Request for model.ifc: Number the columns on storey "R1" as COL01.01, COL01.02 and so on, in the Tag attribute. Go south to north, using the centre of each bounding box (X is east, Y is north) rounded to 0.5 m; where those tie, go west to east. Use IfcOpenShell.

First a look at what the model holds.

```python
import ifcopenshell
import ifcopenshell.util.element
import ifcopenshell.util.placement

model = ifcopenshell.open("model.ifc")
print(model.schema)
storey = next(s for s in model.by_type("IfcBuildingStorey") if s.Name == "R1")
columns = [e for e in ifcopenshell.util.element.get_decomposition(storey) if e.is_a("IfcColumn")]
for e in sorted(columns, key=lambda e: e.id()):
    origin = ifcopenshell.util.placement.get_local_placement(e.ObjectPlacement)[:3, 3]
    print(e.id(), e.Tag, e.Name, origin.round(2) + 0.0, sep=" | ")
```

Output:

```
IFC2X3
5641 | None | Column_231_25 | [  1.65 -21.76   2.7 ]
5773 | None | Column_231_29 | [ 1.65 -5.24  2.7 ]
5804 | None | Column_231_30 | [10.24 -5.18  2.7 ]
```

```python
import ifcopenshell
import ifcopenshell.geom
import ifcopenshell.util.element
import ifcopenshell.util.shape

model = ifcopenshell.open("model.ifc")
settings = ifcopenshell.geom.settings()
settings.set("use-world-coords", True)


def centre(element):
    shape = ifcopenshell.geom.create_shape(settings, element)
    return ifcopenshell.util.shape.get_bbox_centroid(shape.geometry)


storey = next(s for s in model.by_type("IfcBuildingStorey") if s.Name == "R1")
columns = [e for e in ifcopenshell.util.element.get_decomposition(storey) if e.is_a("IfcColumn")]

# Insertion points can sit at a corner or the storey origin, so sort by the geometry (in metres).
centres = {e: centre(e) for e in columns}
columns.sort(key=lambda e: (round(centres[e][1] / 0.5), centres[e][0]))

for i, e in enumerate(columns, start=1):
    number = f"COL01.{i:02d}"
    e.Tag = number
    print(e.id(), number)

model.write("model-out.ifc")
```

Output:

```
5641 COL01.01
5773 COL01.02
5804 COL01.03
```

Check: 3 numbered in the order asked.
